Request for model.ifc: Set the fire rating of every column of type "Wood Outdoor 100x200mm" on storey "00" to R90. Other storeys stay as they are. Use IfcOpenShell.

First a look at what the model holds.

```python
import ifcopenshell
import ifcopenshell.util.element

model = ifcopenshell.open("model.ifc")
print(model.schema)
storey = next(s for s in model.by_type("IfcBuildingStorey") if s.Name == "00")
columns = [e for e in ifcopenshell.util.element.get_decomposition(storey) if e.is_a("IfcColumn")]
seen = {}
for e in columns:
    element_type = ifcopenshell.util.element.get_type(e)
    key = (element_type.Name if element_type != e and element_type else None, ifcopenshell.util.element.get_pset(e, "Pset_ColumnCommon", "FireRating"))
    seen[key] = seen.get(key, 0) + 1
for (name, value), count in sorted(seen.items(), key=str):
    print(count, "x", name, "|", value)
```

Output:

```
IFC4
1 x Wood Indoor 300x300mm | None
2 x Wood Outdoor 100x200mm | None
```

```python
import ifcopenshell
import ifcopenshell.api.pset
import ifcopenshell.util.element

model = ifcopenshell.open("model.ifc")

storey = next(s for s in model.by_type("IfcBuildingStorey") if s.Name == "00")
columns = [e for e in ifcopenshell.util.element.get_decomposition(storey) if e.is_a("IfcColumn")]

count = 0
for e in columns:
    element_type = ifcopenshell.util.element.get_type(e)
    if element_type in (None, e) or element_type.Name != "Wood Outdoor 100x200mm":
        continue
    # add_pset returns the element's existing set when there is one.
    pset = ifcopenshell.api.pset.add_pset(model, product=e, name="Pset_ColumnCommon")
    ifcopenshell.api.pset.edit_pset(model, pset=pset, properties={"FireRating": "R90"})
    count += 1

print(count, "columns updated")

model.write("model_updated.ifc")
```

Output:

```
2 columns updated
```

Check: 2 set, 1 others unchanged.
